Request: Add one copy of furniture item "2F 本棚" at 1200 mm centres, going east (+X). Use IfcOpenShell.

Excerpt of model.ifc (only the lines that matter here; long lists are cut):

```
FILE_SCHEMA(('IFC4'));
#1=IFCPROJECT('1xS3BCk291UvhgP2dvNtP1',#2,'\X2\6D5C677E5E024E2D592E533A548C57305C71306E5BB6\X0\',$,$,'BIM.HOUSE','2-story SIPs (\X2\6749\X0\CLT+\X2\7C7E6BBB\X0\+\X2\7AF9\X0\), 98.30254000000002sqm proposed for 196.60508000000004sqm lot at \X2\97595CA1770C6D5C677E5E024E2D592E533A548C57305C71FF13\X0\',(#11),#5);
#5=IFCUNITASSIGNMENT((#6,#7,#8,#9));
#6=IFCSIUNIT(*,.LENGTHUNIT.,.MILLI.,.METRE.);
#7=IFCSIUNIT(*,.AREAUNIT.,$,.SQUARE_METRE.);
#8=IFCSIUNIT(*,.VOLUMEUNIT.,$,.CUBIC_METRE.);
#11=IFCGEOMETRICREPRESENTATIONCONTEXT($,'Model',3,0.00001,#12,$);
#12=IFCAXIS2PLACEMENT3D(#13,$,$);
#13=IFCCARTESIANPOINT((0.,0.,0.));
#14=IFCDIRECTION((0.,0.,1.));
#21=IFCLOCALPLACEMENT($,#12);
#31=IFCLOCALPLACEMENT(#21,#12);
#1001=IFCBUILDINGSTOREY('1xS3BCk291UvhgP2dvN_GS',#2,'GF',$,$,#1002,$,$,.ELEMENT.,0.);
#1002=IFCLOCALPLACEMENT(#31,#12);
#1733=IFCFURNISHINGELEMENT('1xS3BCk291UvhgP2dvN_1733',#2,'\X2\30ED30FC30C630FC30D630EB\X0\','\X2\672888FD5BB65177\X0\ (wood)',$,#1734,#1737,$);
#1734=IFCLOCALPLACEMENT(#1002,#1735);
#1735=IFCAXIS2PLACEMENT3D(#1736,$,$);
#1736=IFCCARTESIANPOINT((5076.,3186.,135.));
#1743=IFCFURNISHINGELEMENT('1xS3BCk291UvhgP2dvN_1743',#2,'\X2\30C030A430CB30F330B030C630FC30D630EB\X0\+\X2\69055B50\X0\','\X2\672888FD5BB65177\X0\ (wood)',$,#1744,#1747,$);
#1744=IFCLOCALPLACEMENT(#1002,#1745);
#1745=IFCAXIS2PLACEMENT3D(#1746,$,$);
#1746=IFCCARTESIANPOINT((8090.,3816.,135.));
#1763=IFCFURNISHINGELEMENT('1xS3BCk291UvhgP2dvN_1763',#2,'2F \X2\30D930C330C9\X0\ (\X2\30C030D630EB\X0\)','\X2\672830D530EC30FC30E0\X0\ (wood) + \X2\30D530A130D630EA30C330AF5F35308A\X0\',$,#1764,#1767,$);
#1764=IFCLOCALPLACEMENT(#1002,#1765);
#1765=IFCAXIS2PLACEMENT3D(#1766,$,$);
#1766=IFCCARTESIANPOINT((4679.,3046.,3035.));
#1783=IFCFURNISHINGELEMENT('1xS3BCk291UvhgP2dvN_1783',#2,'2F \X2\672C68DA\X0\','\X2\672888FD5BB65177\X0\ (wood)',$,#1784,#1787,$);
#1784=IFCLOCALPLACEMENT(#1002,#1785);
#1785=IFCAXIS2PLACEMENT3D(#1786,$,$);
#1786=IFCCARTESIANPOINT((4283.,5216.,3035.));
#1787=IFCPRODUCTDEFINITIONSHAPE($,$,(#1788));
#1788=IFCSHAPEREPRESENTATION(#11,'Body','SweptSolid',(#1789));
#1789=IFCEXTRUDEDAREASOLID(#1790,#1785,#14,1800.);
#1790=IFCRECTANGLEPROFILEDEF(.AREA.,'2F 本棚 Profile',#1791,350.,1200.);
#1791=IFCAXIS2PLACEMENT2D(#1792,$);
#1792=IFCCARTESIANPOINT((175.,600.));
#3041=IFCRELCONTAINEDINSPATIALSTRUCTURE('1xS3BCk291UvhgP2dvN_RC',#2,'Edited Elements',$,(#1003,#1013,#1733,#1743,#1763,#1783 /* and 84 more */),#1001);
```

```python
import numpy as np
import ifcopenshell
import ifcopenshell.api.geometry
import ifcopenshell.api.root
import ifcopenshell.util.element
import ifcopenshell.util.placement

model = ifcopenshell.open("model.ifc")


def reuse_history(source, copy):
    """copy_class also copies each property set's owner history, people and application; keep the originals."""
    for rel in copy.IsDefinedBy:
        if rel.is_a("IfcRelDefinesByProperties") and (history := rel.RelatingPropertyDefinition.OwnerHistory):
            rel.RelatingPropertyDefinition.OwnerHistory = source.OwnerHistory
            ifcopenshell.util.element.remove_deep2(model, history)


source = model.by_guid("1xS3BCk291UvhgP2dvN_1783")
base = ifcopenshell.util.placement.get_local_placement(source.ObjectPlacement)
step = np.array([1.0, 0.0, 0.0]) * 1200.0

for i in range(1, 2):
    copy = ifcopenshell.api.root.copy_class(model, product=source)
    copy.Representation = ifcopenshell.util.element.copy_deep(
        model, source.Representation, exclude=["IfcGeometricRepresentationContext", "IfcRepresentationMap"]
    )
    reuse_history(source, copy)
    matrix = base.copy()
    matrix[:3, 3] += i * step
    print("added at", matrix[:3, 3].round(3) + 0.0)
    ifcopenshell.api.geometry.edit_object_placement(model, product=copy, matrix=matrix, is_si=False)

model.write("model_updated.ifc")
```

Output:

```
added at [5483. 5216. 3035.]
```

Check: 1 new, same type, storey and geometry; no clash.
